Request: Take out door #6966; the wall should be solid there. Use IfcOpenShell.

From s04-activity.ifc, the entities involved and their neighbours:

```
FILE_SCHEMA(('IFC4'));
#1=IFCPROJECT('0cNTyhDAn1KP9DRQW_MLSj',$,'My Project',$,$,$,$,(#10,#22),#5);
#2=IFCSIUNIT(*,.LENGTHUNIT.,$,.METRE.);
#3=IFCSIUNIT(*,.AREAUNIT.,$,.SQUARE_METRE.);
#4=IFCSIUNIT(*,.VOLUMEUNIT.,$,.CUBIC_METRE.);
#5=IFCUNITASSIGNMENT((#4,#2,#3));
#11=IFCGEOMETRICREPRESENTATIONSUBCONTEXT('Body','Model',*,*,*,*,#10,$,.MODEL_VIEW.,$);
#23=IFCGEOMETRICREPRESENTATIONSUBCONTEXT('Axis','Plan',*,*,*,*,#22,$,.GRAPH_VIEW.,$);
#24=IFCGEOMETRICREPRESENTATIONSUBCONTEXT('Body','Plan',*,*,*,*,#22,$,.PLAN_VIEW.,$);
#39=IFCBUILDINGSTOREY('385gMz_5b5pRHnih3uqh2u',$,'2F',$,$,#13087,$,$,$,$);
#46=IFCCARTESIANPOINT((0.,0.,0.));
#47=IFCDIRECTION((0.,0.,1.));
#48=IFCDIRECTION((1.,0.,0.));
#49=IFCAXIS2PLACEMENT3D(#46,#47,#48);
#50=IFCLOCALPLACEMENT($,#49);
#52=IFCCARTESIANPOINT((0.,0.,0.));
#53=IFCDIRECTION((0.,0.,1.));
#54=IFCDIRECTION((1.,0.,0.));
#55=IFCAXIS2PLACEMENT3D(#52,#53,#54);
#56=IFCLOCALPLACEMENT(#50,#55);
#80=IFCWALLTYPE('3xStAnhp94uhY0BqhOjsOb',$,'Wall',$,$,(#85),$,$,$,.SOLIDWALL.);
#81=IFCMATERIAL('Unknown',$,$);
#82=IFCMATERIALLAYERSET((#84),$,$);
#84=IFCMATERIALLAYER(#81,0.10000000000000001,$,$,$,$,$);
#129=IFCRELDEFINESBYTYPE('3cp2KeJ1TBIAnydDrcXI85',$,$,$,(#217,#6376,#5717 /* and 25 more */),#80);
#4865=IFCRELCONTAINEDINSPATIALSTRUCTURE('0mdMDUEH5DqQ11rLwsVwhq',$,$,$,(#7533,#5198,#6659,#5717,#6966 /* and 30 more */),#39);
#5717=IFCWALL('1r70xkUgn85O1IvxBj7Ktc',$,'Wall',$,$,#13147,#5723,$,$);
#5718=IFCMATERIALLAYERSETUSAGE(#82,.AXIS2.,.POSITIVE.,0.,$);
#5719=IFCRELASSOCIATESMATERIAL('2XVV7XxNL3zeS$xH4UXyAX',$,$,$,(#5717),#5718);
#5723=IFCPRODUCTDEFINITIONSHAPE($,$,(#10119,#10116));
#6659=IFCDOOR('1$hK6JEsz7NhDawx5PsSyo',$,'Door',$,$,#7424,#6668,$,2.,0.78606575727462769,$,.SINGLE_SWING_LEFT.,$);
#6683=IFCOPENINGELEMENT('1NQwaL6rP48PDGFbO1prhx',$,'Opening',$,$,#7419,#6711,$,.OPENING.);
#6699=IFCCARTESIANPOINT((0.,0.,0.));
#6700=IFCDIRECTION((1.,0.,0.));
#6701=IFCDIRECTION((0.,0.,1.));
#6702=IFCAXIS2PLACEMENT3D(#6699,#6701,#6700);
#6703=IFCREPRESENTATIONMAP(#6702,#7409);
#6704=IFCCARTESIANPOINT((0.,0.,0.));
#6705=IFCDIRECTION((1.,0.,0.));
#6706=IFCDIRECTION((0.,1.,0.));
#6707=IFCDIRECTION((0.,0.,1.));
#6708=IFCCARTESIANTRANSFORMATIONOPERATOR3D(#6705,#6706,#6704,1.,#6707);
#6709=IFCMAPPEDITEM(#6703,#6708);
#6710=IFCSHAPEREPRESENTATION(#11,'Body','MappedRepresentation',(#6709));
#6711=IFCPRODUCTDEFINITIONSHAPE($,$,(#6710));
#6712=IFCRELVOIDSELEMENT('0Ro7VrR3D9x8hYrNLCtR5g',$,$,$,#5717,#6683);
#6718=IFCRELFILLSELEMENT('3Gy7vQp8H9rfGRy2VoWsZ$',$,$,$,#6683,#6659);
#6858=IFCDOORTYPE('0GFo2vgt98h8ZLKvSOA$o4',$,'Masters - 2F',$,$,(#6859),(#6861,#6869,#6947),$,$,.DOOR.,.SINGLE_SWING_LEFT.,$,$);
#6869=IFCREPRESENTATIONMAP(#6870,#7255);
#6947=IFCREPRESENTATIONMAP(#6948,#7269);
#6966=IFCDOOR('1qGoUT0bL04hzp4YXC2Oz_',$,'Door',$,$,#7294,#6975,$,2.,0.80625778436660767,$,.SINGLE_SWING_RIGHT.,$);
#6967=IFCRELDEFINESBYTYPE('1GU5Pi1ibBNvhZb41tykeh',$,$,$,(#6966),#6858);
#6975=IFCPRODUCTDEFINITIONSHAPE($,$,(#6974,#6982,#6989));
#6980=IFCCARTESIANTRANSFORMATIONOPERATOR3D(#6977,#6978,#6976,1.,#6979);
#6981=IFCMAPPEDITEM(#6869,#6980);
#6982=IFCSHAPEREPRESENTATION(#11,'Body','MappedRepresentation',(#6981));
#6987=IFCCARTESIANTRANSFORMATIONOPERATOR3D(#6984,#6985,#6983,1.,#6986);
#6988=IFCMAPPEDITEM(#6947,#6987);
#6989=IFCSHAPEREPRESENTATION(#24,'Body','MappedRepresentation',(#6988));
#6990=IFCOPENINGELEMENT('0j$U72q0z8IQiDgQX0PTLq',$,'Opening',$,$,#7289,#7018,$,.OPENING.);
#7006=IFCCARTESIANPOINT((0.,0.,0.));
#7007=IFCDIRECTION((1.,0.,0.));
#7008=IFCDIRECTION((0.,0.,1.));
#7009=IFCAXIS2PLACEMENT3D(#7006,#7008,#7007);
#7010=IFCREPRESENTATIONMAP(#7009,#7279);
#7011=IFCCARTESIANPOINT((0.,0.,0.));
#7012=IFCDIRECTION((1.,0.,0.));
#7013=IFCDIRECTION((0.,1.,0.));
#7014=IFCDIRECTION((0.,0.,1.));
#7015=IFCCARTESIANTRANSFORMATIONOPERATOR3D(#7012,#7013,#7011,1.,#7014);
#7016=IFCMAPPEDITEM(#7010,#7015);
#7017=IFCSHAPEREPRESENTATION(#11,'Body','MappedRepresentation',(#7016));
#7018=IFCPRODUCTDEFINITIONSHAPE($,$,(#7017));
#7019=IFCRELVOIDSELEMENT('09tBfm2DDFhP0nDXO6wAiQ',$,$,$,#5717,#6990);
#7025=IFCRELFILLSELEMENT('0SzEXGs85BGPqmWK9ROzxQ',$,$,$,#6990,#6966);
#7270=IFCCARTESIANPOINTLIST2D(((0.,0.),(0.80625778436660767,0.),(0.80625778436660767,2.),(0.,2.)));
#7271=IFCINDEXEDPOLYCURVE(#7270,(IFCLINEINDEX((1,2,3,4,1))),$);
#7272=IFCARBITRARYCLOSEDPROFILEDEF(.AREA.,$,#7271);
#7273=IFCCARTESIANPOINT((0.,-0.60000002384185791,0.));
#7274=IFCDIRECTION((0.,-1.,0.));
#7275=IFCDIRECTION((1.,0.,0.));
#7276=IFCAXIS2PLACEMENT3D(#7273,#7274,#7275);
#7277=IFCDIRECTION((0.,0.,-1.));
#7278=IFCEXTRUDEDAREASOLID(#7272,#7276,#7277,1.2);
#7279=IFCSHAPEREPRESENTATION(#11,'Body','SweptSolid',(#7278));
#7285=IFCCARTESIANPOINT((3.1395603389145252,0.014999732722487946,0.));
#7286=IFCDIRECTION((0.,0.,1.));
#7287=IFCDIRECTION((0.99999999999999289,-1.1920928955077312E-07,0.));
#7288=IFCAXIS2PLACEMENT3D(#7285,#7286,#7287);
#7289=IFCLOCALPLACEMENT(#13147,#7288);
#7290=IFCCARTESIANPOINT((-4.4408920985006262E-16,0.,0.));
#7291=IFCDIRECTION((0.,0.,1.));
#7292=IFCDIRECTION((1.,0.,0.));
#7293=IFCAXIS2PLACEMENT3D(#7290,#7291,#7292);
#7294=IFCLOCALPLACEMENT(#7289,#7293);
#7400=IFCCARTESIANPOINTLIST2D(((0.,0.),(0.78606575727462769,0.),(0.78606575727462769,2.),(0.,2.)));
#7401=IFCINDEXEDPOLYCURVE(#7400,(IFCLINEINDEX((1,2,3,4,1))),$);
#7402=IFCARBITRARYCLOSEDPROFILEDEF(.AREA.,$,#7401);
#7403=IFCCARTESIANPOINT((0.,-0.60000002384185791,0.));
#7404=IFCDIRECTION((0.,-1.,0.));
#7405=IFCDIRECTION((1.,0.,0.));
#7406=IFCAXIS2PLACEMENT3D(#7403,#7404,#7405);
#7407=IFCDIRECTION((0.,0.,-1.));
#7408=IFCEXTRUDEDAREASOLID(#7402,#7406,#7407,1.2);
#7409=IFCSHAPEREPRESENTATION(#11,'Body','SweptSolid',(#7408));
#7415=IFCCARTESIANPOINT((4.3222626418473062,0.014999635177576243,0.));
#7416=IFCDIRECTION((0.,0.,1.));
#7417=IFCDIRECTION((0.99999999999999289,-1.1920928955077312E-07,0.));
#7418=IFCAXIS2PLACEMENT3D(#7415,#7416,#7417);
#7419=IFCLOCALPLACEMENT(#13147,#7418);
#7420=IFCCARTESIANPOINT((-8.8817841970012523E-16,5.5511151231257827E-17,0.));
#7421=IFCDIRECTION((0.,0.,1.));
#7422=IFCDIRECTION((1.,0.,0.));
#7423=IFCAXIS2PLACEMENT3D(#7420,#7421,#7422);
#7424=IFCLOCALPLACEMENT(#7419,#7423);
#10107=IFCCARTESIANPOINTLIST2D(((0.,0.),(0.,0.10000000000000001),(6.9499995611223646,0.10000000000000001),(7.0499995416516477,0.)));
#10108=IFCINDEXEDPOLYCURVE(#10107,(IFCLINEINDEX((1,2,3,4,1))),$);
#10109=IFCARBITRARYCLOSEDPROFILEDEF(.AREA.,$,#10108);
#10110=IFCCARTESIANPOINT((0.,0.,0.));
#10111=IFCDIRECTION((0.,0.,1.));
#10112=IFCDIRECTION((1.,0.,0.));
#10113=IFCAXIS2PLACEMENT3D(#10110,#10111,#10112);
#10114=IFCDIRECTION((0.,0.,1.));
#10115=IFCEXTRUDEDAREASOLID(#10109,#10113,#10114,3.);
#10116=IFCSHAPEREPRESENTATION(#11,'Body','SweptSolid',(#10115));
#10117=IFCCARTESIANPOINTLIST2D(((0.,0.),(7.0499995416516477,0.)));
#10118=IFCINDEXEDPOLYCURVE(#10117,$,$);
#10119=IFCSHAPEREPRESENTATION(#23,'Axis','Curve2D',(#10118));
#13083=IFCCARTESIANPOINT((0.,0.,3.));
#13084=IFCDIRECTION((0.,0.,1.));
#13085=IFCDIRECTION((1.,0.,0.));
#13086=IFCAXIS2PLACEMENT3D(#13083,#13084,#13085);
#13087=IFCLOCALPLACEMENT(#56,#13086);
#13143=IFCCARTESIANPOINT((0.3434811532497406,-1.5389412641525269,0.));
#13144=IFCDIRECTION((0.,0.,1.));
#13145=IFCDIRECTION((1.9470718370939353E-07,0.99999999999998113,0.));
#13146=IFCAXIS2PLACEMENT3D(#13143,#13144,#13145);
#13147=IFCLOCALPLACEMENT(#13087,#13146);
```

```python
import ifcopenshell
import ifcopenshell.api.feature
import ifcopenshell.api.root
import ifcopenshell.geom
import ifcopenshell.util.shape

model = ifcopenshell.open("s04-activity.ifc")
settings = ifcopenshell.geom.settings()


def volume(element):
    """Net volume in cubic metres, openings subtracted."""
    shape = ifcopenshell.geom.create_shape(settings, element)
    return ifcopenshell.util.shape.get_volume(shape.geometry)


door = model.by_id(6966)
opening = door.FillsVoids[0].RelatingOpeningElement
wall = opening.VoidsElements[0].RelatingBuildingElement
before = volume(wall)

ifcopenshell.api.root.remove_product(model, product=door)
ifcopenshell.api.feature.remove_feature(model, feature=opening)

after = volume(wall)

print(f"wall volume {before:.3f} -> {after:.3f} m3")

model.write("s04-activity-out.ifc")
```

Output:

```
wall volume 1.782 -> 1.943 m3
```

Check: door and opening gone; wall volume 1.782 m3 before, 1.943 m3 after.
